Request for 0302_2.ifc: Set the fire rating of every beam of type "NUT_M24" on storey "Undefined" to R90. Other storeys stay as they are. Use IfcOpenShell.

First a look at what the model holds.

```python
import ifcopenshell
import ifcopenshell.util.element

model = ifcopenshell.open("0302_2.ifc")
print(model.schema)
storey = next(s for s in model.by_type("IfcBuildingStorey") if s.Name == "Undefined")
beams = [e for e in ifcopenshell.util.element.get_decomposition(storey) if e.is_a("IfcBeam")]
seen = {}
for e in beams:
    element_type = ifcopenshell.util.element.get_type(e)
    key = (element_type.Name if element_type != e and element_type else None, ifcopenshell.util.element.get_pset(e, "Pset_BeamCommon", "FireRating"))
    seen[key] = seen.get(key, 0) + 1
for (name, value), count in sorted(seen.items(), key=str):
    print(count, "x", name, "|", value)
```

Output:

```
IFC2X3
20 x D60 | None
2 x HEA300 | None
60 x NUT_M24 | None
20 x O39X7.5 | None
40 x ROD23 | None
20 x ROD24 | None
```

```python
import ifcopenshell
import ifcopenshell.api.pset
import ifcopenshell.util.element

model = ifcopenshell.open("0302_2.ifc")

storey = next(s for s in model.by_type("IfcBuildingStorey") if s.Name == "Undefined")
beams = [e for e in ifcopenshell.util.element.get_decomposition(storey) if e.is_a("IfcBeam")]

count = 0
for e in beams:
    element_type = ifcopenshell.util.element.get_type(e)
    if element_type in (None, e) or element_type.Name != "NUT_M24":
        continue
    found = ifcopenshell.util.element.get_pset(e, "Pset_BeamCommon", should_inherit=False)
    if found:
        pset = model.by_id(found["id"])
        if len(ifcopenshell.util.element.get_elements_by_pset(pset)) > 1:
            pset = ifcopenshell.api.pset.unshare_pset(model, products=[e], pset=pset)[0]
    else:
        pset = ifcopenshell.api.pset.add_pset(model, product=e, name="Pset_BeamCommon")
    ifcopenshell.api.pset.edit_pset(model, pset=pset, properties={"FireRating": "R90"})
    count += 1

print(count, "beams updated")

model.write("0302_2_rev.ifc")
```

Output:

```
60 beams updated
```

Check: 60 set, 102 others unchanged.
